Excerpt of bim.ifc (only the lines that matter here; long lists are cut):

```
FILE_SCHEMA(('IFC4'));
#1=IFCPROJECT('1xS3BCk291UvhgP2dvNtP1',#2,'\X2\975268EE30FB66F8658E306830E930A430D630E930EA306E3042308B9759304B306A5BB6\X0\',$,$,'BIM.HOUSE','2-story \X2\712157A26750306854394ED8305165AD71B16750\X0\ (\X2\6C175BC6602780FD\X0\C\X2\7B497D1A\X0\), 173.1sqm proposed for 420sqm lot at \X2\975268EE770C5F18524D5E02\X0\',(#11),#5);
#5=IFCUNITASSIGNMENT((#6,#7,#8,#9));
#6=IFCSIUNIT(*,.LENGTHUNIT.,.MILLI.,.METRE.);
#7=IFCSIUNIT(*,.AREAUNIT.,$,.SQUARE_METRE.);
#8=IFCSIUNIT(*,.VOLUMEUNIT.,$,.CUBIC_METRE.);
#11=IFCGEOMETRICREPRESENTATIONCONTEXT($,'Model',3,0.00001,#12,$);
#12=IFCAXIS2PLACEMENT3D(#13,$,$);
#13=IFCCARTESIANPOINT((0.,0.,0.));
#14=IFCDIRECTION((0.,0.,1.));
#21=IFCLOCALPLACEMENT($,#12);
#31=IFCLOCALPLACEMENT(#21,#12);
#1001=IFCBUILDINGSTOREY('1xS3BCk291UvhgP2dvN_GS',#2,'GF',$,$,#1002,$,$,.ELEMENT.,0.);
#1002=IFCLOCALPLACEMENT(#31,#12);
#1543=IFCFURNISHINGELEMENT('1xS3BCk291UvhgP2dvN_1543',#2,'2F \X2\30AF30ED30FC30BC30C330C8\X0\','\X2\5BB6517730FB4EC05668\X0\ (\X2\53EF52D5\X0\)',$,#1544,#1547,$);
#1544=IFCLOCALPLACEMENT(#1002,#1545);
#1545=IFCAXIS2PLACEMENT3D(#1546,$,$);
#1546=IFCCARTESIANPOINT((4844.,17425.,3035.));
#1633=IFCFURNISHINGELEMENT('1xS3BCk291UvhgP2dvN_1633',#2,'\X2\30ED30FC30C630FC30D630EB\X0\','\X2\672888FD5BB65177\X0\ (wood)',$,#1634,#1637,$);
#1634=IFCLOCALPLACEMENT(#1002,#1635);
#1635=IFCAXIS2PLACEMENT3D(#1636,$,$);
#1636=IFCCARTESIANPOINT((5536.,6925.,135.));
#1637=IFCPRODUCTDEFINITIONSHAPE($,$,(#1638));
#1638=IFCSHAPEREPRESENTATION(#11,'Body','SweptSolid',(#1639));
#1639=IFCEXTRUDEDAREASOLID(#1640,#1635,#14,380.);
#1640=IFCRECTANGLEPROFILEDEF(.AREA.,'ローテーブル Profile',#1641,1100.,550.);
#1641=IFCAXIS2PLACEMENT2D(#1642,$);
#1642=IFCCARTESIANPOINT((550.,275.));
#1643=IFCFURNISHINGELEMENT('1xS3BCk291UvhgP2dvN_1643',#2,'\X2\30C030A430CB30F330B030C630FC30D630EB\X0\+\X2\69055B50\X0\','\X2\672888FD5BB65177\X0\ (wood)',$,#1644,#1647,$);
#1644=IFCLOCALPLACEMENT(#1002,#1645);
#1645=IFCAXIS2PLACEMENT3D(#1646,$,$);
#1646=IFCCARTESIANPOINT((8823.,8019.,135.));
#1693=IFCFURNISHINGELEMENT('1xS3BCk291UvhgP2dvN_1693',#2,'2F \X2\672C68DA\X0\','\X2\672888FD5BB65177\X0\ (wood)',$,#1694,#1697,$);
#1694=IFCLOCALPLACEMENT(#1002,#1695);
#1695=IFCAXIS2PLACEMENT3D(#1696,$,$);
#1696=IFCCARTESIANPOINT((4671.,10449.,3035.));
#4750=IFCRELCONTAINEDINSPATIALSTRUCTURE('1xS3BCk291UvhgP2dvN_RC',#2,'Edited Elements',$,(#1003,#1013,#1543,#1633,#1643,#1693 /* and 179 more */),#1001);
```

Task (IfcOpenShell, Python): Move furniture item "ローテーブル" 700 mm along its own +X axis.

```python
import ifcopenshell
import ifcopenshell.api.geometry
import ifcopenshell.util.placement

model = ifcopenshell.open("bim.ifc")

item = model.by_id(1633)
matrix = ifcopenshell.util.placement.get_local_placement(item.ObjectPlacement)
matrix[:3, 3] += matrix[:3, 0] * 700.0
ifcopenshell.api.geometry.edit_object_placement(model, product=item, matrix=matrix, is_si=False)

print(ifcopenshell.util.placement.get_local_placement(item.ObjectPlacement).round(3) + 0.0)

model.write("bim_updated.ifc")
```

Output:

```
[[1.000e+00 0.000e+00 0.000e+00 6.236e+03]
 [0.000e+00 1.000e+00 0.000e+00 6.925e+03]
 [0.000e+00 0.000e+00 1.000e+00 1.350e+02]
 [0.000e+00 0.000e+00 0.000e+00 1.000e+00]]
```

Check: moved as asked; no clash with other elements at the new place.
